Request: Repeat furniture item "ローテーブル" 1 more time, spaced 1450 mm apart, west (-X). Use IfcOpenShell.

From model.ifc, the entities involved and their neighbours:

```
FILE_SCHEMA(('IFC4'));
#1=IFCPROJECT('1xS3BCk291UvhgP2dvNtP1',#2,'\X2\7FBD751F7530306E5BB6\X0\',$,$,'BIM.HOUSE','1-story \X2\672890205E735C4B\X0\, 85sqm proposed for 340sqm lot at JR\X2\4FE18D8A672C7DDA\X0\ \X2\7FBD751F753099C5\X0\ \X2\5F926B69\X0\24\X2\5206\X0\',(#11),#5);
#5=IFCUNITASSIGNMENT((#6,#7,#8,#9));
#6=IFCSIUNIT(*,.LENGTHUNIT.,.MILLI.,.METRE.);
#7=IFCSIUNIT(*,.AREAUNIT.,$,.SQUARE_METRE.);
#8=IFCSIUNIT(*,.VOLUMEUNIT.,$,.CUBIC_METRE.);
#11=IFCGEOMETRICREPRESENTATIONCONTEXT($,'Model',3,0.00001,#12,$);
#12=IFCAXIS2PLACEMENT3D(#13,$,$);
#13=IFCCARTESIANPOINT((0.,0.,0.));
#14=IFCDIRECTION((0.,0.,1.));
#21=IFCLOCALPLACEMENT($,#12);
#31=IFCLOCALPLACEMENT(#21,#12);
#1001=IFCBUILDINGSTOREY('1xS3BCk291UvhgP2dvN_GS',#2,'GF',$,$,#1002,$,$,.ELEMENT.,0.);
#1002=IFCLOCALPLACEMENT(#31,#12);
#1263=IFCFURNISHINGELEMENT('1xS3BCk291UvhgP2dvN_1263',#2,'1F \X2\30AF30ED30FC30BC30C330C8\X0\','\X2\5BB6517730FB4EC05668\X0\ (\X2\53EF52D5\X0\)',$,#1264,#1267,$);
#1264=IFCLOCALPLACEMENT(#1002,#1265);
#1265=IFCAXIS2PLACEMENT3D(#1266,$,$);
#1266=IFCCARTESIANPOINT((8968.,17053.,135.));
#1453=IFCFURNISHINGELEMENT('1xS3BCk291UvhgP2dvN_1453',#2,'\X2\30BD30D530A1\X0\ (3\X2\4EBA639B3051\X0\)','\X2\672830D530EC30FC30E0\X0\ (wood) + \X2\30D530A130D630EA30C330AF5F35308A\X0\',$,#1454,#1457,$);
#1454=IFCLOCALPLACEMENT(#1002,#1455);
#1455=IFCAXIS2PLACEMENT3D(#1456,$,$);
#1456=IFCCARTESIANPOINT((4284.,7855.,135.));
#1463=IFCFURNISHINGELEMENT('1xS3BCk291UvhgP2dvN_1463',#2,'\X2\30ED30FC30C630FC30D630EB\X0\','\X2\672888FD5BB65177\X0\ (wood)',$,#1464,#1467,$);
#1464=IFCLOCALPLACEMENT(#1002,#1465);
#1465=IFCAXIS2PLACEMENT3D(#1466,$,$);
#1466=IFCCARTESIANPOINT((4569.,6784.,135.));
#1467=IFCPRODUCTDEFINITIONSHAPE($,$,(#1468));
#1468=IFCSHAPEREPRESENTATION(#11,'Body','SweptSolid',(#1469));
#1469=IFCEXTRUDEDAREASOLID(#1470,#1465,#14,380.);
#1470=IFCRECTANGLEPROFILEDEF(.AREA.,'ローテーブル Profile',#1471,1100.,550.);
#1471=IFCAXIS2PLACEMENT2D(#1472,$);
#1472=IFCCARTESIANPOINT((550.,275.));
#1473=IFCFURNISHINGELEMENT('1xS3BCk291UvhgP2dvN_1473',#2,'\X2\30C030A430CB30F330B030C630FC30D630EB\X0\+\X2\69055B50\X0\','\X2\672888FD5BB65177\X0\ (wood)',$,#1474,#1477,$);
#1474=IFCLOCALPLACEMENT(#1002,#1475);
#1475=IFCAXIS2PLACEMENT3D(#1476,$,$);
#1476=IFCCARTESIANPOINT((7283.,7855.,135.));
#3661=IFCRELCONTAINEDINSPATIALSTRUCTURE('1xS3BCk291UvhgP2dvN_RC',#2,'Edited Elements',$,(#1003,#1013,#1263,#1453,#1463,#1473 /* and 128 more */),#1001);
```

```python
import numpy as np
import ifcopenshell
import ifcopenshell.api.geometry
import ifcopenshell.api.root
import ifcopenshell.util.element
import ifcopenshell.util.placement

model = ifcopenshell.open("model.ifc")


def reuse_history(source, copy):
    """copy_class also copies each property set's owner history, people and application; keep the originals."""
    for rel in copy.IsDefinedBy:
        if rel.is_a("IfcRelDefinesByProperties") and (history := rel.RelatingPropertyDefinition.OwnerHistory):
            rel.RelatingPropertyDefinition.OwnerHistory = source.OwnerHistory
            ifcopenshell.util.element.remove_deep2(model, history)


source = model.by_id(1463)
base = ifcopenshell.util.placement.get_local_placement(source.ObjectPlacement)
step = np.array([-1.0, 0.0, 0.0]) * 1450.0

for i in range(1, 2):
    copy = ifcopenshell.api.root.copy_class(model, product=source)
    copy.Representation = ifcopenshell.util.element.copy_deep(
        model, source.Representation, exclude=["IfcGeometricRepresentationContext", "IfcRepresentationMap"]
    )
    reuse_history(source, copy)
    matrix = base.copy()
    matrix[:3, 3] += i * step
    print("added at", matrix[:3, 3].round(3) + 0.0)
    ifcopenshell.api.geometry.edit_object_placement(model, product=copy, matrix=matrix, is_si=False)

model.write("model-out.ifc")
```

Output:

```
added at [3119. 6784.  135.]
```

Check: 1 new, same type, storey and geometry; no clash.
